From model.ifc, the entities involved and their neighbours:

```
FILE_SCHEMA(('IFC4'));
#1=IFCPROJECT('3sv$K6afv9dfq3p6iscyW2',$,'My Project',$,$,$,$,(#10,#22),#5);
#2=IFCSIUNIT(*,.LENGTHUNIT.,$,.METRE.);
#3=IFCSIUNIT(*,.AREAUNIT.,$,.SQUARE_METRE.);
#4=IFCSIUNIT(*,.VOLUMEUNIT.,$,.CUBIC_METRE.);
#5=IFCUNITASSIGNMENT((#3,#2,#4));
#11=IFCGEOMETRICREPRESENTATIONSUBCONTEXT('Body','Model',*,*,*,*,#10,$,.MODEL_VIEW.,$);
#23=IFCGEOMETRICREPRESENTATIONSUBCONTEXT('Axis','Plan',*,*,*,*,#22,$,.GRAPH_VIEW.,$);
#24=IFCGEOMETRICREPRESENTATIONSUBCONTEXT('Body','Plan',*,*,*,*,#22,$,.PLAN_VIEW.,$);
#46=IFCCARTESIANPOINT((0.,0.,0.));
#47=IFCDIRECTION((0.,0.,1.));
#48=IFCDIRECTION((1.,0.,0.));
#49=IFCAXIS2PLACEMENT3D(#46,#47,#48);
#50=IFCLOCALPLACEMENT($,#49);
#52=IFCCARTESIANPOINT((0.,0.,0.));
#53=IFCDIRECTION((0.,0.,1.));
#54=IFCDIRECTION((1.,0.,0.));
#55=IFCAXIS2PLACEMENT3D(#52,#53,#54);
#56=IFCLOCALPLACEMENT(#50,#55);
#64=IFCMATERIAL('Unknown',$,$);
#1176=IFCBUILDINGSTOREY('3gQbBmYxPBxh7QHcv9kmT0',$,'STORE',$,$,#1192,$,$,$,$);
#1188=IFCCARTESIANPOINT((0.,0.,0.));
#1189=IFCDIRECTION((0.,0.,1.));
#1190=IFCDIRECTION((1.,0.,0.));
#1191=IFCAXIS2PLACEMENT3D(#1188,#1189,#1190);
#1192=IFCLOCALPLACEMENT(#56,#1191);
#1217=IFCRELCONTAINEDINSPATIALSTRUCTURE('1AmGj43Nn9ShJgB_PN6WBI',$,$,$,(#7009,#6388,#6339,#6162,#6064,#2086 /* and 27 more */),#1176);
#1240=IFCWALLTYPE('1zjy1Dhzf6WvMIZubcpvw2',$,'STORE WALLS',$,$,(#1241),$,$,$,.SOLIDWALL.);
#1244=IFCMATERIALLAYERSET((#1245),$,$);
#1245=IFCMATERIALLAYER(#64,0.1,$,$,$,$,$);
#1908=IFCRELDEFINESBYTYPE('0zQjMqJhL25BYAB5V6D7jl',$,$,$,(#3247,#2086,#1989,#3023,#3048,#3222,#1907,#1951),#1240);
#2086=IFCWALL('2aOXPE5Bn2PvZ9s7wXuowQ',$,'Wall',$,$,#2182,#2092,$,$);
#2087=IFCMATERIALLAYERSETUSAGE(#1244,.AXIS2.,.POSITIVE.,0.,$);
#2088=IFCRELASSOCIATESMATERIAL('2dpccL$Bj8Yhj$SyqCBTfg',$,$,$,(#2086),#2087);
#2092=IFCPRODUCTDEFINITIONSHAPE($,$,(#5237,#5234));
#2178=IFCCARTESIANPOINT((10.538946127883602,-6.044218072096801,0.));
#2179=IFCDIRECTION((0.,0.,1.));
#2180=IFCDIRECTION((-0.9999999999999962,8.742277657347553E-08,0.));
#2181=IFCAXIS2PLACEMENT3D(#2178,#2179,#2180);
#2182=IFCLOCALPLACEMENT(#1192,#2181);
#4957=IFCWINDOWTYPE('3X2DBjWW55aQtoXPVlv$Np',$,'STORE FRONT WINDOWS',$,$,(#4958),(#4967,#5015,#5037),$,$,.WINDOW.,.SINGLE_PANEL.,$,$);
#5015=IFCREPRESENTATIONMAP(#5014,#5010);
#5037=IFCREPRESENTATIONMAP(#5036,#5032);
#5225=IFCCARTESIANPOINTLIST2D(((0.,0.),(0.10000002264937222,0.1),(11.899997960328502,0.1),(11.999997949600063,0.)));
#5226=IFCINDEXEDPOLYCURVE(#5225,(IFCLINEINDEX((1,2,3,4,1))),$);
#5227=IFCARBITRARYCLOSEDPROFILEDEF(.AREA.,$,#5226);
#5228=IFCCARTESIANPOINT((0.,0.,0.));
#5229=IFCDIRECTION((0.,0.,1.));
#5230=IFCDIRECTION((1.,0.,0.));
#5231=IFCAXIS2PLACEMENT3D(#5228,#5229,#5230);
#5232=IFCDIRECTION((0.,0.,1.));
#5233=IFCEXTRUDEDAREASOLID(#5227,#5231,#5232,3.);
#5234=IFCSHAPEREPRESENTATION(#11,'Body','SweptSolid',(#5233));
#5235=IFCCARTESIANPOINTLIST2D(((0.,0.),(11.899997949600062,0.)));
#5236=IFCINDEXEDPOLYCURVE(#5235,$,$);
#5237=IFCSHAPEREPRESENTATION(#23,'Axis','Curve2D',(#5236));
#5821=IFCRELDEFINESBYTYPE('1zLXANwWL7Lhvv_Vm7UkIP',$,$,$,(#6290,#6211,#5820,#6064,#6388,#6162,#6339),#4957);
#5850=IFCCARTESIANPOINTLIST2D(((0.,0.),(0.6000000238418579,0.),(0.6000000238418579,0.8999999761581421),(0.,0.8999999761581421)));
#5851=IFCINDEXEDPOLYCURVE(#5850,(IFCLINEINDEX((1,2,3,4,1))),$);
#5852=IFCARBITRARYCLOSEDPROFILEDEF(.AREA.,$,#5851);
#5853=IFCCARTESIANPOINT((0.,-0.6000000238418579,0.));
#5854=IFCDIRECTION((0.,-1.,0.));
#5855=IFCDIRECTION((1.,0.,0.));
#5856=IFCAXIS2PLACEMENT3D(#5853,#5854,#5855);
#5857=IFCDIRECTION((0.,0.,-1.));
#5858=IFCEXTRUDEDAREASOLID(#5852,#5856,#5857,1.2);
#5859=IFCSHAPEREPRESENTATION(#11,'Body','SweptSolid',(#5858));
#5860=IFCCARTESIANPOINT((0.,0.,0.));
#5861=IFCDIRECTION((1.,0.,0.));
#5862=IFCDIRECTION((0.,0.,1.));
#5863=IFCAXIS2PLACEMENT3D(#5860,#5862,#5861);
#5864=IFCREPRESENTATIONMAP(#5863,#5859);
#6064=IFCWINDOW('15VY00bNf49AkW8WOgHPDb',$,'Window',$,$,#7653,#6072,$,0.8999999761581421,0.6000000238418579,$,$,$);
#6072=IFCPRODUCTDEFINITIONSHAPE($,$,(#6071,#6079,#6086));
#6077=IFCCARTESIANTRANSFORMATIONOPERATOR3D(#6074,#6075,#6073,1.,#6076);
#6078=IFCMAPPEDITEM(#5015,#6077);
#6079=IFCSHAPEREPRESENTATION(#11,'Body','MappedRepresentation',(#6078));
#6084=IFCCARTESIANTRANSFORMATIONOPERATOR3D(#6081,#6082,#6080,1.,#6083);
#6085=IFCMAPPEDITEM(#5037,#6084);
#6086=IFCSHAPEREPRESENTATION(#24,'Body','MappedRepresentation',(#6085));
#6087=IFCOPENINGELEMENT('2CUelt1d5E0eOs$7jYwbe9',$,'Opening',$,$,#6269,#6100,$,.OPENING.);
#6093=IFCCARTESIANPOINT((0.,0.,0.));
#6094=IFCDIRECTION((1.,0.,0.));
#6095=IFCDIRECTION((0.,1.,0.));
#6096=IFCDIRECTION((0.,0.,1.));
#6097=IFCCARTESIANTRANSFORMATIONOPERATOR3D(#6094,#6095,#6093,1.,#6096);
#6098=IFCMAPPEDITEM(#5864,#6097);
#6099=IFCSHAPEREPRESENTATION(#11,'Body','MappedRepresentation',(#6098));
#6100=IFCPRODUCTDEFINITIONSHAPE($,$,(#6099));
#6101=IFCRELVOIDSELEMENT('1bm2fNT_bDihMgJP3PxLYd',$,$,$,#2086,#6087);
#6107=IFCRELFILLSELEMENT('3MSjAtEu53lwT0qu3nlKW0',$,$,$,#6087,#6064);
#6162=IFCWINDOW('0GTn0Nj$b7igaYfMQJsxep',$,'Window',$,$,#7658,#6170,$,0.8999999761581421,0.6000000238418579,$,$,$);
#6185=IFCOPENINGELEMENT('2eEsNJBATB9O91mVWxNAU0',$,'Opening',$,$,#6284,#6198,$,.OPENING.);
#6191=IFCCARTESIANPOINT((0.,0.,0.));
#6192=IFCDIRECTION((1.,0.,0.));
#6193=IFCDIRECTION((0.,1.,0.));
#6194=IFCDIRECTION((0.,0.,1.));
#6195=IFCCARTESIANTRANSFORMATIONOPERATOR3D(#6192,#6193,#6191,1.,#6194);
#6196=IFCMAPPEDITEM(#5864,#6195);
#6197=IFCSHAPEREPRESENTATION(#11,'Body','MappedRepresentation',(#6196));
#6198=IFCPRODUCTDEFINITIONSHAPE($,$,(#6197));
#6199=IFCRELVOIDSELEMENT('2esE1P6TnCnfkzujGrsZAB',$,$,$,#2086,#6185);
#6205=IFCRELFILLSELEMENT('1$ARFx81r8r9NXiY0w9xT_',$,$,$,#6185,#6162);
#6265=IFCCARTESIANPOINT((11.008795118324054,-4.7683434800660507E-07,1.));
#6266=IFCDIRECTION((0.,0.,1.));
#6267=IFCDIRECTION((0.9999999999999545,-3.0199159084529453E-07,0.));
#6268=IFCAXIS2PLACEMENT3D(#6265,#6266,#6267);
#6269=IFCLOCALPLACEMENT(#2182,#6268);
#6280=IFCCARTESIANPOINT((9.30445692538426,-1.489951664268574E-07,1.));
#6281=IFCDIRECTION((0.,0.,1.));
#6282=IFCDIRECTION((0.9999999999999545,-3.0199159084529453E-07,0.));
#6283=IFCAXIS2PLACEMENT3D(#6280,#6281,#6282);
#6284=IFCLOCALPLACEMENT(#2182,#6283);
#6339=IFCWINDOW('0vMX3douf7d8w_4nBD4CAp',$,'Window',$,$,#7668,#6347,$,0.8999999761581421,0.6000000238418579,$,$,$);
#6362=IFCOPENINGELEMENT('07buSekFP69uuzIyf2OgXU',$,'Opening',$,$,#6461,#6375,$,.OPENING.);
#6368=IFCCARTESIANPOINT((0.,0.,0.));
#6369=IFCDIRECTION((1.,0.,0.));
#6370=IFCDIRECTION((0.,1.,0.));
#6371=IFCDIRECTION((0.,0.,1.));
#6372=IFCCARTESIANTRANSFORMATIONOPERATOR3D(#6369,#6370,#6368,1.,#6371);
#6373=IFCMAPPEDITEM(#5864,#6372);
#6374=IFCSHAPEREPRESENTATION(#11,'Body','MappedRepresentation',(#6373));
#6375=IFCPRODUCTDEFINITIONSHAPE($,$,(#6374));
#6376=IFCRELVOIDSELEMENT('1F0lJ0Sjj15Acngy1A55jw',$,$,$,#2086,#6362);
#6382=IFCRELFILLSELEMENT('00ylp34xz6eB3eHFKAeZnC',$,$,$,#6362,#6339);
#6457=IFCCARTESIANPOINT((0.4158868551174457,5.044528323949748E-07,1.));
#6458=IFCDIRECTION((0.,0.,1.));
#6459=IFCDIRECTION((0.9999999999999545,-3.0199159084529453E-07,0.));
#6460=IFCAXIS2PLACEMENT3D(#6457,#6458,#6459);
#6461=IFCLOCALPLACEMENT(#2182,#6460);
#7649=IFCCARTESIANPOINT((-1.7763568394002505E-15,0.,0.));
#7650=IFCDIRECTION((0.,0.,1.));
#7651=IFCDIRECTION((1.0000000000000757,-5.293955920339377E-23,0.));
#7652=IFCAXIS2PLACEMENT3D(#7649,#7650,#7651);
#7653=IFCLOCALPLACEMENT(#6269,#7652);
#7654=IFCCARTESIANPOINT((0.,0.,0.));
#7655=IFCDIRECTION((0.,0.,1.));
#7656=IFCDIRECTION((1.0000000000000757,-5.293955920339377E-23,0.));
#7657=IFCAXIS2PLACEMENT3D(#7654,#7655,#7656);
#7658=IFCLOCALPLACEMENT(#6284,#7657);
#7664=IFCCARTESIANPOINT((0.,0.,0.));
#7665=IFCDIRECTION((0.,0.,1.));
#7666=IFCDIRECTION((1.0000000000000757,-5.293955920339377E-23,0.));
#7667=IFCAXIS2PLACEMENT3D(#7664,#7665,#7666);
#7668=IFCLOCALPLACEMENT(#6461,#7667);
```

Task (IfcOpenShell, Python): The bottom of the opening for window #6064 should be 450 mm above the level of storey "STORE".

```python
import numpy as np
import ifcopenshell
import ifcopenshell.api.geometry
import ifcopenshell.geom
import ifcopenshell.util.element
import ifcopenshell.util.placement
import ifcopenshell.util.shape
import ifcopenshell.util.unit

model = ifcopenshell.open("model.ifc")
unit_scale = ifcopenshell.util.unit.calculate_unit_scale(model)

window = model.by_guid("15VY00bNf49AkW8WOgHPDb")
opening = window.FillsVoids[0].RelatingOpeningElement
storey = ifcopenshell.util.element.get_container(window, ifc_class="IfcBuildingStorey")
level = ifcopenshell.util.placement.get_local_placement(storey.ObjectPlacement)[2, 3]

# The opening's origin need not be at the sill, so measure its lowest point.
shape = ifcopenshell.geom.create_shape(ifcopenshell.geom.settings(), opening)
bottom = ifcopenshell.util.shape.get_shape_bottom_elevation(shape, shape.geometry) / unit_scale
dz = level + 0.45 - bottom

shift = np.array([0.0, 0.0, dz])
# The window is placed relative to its opening, so it follows when the opening moves.
matrix = ifcopenshell.util.placement.get_local_placement(opening.ObjectPlacement)
matrix[:3, 3] += shift
ifcopenshell.api.geometry.edit_object_placement(
    model, product=opening, matrix=matrix, is_si=False, should_transform_children=True
)

print(f"moved by {dz * unit_scale:+.3f} m")

model.write("model_edited.ifc")
```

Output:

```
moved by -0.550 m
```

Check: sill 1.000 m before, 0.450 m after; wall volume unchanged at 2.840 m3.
